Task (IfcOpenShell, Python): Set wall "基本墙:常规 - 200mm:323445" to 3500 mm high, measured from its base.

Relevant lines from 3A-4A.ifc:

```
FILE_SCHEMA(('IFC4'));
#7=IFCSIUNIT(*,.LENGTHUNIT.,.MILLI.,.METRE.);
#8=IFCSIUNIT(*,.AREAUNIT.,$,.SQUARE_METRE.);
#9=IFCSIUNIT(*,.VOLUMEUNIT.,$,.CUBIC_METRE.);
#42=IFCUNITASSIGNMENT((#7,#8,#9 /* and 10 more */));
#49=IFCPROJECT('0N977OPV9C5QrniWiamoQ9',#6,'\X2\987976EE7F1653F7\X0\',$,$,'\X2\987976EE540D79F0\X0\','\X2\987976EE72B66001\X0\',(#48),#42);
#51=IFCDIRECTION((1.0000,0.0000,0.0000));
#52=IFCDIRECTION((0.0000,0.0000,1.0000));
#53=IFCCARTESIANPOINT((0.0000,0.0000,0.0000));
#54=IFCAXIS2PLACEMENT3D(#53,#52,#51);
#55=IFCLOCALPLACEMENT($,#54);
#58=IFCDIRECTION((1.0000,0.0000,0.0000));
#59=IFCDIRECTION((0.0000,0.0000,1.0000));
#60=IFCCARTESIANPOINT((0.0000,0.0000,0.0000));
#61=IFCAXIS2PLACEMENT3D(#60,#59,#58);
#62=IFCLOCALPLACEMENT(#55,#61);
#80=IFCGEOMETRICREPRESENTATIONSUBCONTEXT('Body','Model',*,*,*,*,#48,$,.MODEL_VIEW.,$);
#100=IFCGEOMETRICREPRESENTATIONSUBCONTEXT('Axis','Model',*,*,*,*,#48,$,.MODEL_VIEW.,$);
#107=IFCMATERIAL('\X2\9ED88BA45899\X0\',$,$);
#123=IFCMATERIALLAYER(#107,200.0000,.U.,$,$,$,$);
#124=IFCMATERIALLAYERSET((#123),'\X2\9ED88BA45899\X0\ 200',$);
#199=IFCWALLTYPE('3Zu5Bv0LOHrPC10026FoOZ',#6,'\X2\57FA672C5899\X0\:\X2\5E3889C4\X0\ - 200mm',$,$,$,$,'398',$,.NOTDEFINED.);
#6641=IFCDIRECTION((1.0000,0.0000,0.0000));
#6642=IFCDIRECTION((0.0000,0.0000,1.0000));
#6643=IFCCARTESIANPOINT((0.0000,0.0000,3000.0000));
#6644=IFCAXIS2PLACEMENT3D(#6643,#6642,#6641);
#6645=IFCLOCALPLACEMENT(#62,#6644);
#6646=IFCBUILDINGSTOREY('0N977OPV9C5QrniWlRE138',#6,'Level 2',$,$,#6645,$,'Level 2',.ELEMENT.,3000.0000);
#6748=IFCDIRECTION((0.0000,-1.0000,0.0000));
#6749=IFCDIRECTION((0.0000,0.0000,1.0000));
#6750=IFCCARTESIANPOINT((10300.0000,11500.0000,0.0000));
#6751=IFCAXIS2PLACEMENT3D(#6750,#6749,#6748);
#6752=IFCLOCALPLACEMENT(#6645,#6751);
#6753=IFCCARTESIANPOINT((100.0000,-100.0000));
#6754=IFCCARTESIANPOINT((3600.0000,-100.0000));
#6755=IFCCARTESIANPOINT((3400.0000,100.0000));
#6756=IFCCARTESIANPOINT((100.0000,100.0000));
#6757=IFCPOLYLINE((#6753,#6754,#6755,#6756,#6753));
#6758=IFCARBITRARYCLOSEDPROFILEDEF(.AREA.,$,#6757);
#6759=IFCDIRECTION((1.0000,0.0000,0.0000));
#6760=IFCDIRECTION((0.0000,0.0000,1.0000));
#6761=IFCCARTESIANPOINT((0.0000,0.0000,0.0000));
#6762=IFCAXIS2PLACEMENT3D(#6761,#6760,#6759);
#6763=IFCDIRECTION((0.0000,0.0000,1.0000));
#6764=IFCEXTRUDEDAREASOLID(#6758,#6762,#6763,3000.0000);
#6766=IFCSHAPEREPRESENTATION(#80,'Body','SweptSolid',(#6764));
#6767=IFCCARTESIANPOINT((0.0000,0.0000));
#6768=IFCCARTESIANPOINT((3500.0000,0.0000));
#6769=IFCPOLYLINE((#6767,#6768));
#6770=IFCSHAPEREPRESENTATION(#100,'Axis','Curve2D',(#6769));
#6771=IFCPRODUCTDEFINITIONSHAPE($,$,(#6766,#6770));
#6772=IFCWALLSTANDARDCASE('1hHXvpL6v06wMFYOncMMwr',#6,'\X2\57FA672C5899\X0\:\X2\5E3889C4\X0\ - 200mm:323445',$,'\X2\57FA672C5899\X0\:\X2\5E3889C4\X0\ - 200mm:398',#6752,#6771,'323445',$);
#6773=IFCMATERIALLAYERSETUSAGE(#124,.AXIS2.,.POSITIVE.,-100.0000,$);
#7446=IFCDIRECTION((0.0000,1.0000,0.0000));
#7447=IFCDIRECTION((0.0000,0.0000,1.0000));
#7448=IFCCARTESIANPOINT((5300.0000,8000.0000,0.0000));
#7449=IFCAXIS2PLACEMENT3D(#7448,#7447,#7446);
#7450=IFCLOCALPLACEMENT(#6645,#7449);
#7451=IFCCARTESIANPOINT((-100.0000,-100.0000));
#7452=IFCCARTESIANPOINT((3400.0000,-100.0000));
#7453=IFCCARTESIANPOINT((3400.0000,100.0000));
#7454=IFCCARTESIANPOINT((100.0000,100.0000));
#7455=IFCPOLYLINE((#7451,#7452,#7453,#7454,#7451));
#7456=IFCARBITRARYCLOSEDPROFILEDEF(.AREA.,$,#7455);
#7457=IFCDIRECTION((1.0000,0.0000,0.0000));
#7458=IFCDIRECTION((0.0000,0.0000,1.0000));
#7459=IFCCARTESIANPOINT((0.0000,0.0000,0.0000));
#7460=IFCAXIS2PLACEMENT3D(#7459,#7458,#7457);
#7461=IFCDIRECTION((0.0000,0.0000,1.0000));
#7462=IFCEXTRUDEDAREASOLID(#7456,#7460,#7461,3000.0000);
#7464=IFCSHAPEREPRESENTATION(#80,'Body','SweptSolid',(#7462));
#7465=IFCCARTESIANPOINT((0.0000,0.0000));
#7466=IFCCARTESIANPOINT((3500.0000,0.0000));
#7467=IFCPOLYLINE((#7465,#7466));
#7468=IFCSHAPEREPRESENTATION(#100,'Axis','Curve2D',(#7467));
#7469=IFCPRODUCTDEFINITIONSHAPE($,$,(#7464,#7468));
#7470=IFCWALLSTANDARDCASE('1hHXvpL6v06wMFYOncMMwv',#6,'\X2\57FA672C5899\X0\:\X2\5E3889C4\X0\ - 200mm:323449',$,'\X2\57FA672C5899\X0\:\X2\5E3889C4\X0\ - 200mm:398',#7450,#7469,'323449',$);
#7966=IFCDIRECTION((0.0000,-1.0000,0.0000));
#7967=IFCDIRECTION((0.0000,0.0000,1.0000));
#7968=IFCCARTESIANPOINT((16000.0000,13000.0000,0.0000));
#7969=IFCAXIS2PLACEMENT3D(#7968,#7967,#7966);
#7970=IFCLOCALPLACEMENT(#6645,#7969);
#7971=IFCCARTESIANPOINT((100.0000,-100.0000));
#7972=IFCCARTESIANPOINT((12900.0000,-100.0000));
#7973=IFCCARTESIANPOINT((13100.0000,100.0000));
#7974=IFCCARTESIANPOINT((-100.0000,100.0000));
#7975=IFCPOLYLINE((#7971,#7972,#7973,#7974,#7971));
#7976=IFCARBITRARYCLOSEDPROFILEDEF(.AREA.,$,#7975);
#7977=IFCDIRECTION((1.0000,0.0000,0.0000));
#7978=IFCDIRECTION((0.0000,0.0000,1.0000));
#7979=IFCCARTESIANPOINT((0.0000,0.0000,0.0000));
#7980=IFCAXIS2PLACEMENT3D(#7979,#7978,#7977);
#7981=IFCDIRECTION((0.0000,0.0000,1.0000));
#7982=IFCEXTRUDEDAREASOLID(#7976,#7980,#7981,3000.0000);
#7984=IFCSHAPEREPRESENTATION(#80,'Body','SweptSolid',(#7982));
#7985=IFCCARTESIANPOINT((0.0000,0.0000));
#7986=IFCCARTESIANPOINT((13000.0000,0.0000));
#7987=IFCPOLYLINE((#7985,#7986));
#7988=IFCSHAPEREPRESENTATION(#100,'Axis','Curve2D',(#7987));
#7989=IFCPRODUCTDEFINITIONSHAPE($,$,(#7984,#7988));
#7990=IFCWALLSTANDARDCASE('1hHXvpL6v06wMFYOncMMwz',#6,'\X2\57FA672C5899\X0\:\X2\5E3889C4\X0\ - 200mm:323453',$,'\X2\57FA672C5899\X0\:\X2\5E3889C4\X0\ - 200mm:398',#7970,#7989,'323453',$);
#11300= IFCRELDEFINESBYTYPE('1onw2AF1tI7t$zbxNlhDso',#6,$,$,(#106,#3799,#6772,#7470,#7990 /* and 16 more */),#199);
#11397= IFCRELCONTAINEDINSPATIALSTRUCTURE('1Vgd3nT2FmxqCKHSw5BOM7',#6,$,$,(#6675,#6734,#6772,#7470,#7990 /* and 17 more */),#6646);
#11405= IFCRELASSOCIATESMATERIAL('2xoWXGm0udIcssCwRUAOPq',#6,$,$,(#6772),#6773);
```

```python
import ifcopenshell
import ifcopenshell.geom
import ifcopenshell.util.representation
import ifcopenshell.util.shape
import ifcopenshell.util.unit

model = ifcopenshell.open("3A-4A.ifc")
unit_scale = ifcopenshell.util.unit.calculate_unit_scale(model)
settings = ifcopenshell.geom.settings()


def volume(element):
    """Net volume in cubic metres, openings subtracted."""
    shape = ifcopenshell.geom.create_shape(settings, element)
    return ifcopenshell.util.shape.get_volume(shape.geometry)


wall = model.by_id(6772)
before = volume(wall)

body = ifcopenshell.util.representation.get_representation(wall, "Model", "Body")
solid = body.Items[0]
old_height = solid.Depth
solid.Depth = 3.5 / unit_scale
after = volume(wall)

print(f"height {old_height:g} -> {solid.Depth:g}, volume {before:.3f} -> {after:.3f} m3")

model.write("3A-4A_edited.ifc")
```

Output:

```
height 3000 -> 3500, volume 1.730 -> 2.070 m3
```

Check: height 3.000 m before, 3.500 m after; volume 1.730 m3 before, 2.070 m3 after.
